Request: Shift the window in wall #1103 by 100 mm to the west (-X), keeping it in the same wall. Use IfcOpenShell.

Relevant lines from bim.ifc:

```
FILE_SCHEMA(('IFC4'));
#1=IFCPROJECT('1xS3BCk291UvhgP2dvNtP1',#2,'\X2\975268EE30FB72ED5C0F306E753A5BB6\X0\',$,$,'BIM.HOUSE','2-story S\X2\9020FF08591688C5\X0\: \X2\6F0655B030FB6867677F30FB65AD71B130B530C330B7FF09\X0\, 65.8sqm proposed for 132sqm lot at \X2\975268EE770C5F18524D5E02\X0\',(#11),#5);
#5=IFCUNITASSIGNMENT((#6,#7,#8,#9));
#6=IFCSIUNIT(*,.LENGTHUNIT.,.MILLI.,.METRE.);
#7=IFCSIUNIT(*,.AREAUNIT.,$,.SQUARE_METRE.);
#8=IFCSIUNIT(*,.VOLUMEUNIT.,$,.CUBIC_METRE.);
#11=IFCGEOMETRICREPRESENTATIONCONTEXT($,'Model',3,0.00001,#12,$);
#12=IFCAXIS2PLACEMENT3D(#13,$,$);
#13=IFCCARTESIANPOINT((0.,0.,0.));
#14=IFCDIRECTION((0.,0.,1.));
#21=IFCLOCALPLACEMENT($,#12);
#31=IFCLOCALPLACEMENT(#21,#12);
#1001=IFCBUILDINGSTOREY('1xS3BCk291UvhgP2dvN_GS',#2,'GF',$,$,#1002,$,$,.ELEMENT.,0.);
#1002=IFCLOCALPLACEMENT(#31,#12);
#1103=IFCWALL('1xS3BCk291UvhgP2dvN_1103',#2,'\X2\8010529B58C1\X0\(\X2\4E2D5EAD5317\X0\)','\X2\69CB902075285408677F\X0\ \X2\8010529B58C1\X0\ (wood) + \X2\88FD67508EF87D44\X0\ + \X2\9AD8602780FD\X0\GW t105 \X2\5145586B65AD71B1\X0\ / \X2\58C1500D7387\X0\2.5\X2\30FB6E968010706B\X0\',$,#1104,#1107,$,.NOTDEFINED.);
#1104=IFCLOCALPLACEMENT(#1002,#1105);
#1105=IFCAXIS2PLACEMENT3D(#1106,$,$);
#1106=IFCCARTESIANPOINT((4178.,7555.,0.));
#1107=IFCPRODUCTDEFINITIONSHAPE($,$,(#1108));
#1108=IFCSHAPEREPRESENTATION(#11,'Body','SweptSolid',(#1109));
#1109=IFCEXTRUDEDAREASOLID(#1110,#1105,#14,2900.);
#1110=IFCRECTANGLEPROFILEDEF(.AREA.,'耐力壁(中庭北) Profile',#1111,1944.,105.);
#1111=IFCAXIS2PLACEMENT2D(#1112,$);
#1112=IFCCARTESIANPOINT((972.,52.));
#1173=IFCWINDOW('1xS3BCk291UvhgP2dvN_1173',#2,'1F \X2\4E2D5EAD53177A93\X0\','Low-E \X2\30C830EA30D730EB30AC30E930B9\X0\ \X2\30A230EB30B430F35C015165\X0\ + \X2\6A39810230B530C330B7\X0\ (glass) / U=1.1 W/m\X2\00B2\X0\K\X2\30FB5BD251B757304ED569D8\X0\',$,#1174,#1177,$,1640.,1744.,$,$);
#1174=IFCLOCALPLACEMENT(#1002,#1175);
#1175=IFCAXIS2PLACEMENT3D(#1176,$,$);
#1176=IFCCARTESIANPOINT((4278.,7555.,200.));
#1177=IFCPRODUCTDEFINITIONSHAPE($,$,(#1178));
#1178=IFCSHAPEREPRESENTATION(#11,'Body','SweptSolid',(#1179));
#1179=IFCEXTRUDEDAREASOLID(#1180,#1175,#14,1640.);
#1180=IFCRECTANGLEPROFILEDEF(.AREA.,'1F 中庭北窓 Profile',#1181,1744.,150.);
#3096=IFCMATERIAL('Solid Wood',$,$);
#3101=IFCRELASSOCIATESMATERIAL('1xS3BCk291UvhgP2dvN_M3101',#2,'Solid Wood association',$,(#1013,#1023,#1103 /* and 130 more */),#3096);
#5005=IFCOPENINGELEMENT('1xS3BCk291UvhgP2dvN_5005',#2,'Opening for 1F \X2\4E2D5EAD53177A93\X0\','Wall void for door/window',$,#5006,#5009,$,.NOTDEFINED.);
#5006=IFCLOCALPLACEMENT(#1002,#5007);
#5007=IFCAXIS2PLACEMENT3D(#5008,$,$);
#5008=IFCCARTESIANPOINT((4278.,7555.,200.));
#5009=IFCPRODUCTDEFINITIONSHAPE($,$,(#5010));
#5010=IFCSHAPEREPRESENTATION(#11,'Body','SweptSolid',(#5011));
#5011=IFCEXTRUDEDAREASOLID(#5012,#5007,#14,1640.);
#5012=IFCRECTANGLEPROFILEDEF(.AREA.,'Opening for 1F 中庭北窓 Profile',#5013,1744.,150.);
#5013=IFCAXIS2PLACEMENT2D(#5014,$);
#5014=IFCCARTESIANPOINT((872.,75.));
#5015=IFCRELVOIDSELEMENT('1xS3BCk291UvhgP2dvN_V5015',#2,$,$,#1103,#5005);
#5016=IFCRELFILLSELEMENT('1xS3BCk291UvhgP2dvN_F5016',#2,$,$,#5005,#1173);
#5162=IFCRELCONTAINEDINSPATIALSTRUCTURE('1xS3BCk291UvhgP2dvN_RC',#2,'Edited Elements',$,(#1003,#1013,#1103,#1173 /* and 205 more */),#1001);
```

```python
import ifcopenshell
import ifcopenshell.api.geometry
import ifcopenshell.util.placement
import ifcopenshell.util.unit

model = ifcopenshell.open("bim.ifc")
unit_scale = ifcopenshell.util.unit.calculate_unit_scale(model)

window = model.by_guid("1xS3BCk291UvhgP2dvN_1173")
opening = window.FillsVoids[0].RelatingOpeningElement
wall = opening.VoidsElements[0].RelatingBuildingElement

wall_matrix = ifcopenshell.util.placement.get_local_placement(wall.ObjectPlacement)
shift = wall_matrix[:3, 0] * -0.1 / unit_scale
before = ifcopenshell.util.placement.get_local_placement(window.ObjectPlacement)[:3, 3].copy()

# The window is not placed relative to its opening, so move both.
for product in (opening, window):
    matrix = ifcopenshell.util.placement.get_local_placement(product.ObjectPlacement)
    matrix[:3, 3] += shift
    ifcopenshell.api.geometry.edit_object_placement(model, product=product, matrix=matrix, is_si=False)

after = ifcopenshell.util.placement.get_local_placement(window.ObjectPlacement)[:3, 3]
print("window moved by", (after - before).round(3) + 0.0)

model.write("bim_v2.ifc")
```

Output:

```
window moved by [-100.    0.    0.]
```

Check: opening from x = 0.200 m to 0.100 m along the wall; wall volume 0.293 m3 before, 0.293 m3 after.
